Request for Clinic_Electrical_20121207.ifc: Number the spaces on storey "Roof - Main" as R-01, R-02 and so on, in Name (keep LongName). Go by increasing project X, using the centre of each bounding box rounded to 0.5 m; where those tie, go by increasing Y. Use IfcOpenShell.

First a look at what the model holds.

```python
import ifcopenshell
import ifcopenshell.util.element
import ifcopenshell.util.placement

model = ifcopenshell.open("Clinic_Electrical_20121207.ifc")
print(model.schema)
storey = next(s for s in model.by_type("IfcBuildingStorey") if s.Name == "Roof - Main")
spaces = [e for e in ifcopenshell.util.element.get_decomposition(storey) if e.is_a("IfcSpace")]
for e in sorted(spaces, key=lambda e: e.id()):
    origin = ifcopenshell.util.placement.get_local_placement(e.ObjectPlacement)[:3, 3]
    print(e.id(), e.Name, e.LongName, origin.round(2) + 0.0, sep=" | ")
```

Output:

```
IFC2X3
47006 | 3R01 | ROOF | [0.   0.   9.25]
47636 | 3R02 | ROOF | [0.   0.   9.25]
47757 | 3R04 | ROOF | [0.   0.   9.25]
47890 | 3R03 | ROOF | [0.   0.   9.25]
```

```python
import ifcopenshell
import ifcopenshell.geom
import ifcopenshell.util.element
import ifcopenshell.util.shape

model = ifcopenshell.open("Clinic_Electrical_20121207.ifc")
settings = ifcopenshell.geom.settings()
settings.set("use-world-coords", True)


def centre(element):
    shape = ifcopenshell.geom.create_shape(settings, element)
    return ifcopenshell.util.shape.get_bbox_centroid(shape.geometry)


storey = next(s for s in model.by_type("IfcBuildingStorey") if s.Name == "Roof - Main")
spaces = [e for e in ifcopenshell.util.element.get_decomposition(storey) if e.is_a("IfcSpace")]

# Insertion points can sit at a corner or the storey origin, so sort by the geometry (in metres).
centres = {e: centre(e) for e in spaces}
spaces.sort(key=lambda e: (round(centres[e][0] / 0.5), centres[e][1]))

for i, e in enumerate(spaces, start=1):
    number = f"R-{i:02d}"
    e.Name = number
    print(e.id(), number)

model.write("Clinic_Electrical_20121207_edited.ifc")
```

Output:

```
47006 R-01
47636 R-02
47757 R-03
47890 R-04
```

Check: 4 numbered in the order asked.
